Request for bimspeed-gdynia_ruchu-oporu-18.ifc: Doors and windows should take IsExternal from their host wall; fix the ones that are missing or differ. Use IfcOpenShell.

First a look at what the model holds.

```python
import ifcopenshell
import ifcopenshell.util.element

model = ifcopenshell.open("bimspeed-gdynia_ruchu-oporu-18.ifc")
print(model.schema)
seen = {}
for e in model.by_type("IfcDoor") + model.by_type("IfcWindow"):
    if not e.FillsVoids:
        continue
    host = e.FillsVoids[0].RelatingOpeningElement.VoidsElements[0].RelatingBuildingElement
    own = ifcopenshell.util.element.get_pset(e, f"Pset_{e.is_a()[3:].removesuffix('StandardCase')}Common", "IsExternal")
    wall = ifcopenshell.util.element.get_pset(host, "Pset_WallCommon", "IsExternal")
    seen[e.is_a(), own, wall] = seen.get((e.is_a(), own, wall), 0) + 1
for (cls, own, wall), count in sorted(seen.items(), key=str):
    print(count, cls, "IsExternal:", own, "| host wall:", wall)
```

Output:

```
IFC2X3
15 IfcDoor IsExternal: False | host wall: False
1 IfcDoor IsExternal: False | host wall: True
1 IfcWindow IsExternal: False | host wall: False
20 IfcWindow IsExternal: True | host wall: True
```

```python
import ifcopenshell
import ifcopenshell.api.pset
import ifcopenshell.util.element

model = ifcopenshell.open("bimspeed-gdynia_ruchu-oporu-18.ifc")

count = 0
for ifc_class, pset_name in (("IfcDoor", "Pset_DoorCommon"), ("IfcWindow", "Pset_WindowCommon")):
    for e in model.by_type(ifc_class):
        if not e.FillsVoids:
            continue
        host = e.FillsVoids[0].RelatingOpeningElement.VoidsElements[0].RelatingBuildingElement
        external = ifcopenshell.util.element.get_pset(host, "Pset_WallCommon", "IsExternal")
        if external is None or ifcopenshell.util.element.get_pset(e, pset_name, "IsExternal") == external:
            continue
        pset = ifcopenshell.api.pset.add_pset(model, product=e, name=pset_name)
        ifcopenshell.api.pset.edit_pset(model, pset=pset, properties={"IsExternal": external})
        count += 1

print(count, "updated")

model.write("bimspeed-gdynia_ruchu-oporu-18_v2.ifc")
```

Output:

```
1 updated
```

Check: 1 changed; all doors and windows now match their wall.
